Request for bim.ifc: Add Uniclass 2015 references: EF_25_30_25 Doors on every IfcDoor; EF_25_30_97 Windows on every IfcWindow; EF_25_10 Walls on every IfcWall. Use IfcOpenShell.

First a look at what the model holds.

```python
import ifcopenshell

model = ifcopenshell.open("bim.ifc")
print(model.schema)
print("classifications:", [c.Name for c in model.by_type("IfcClassification")])
for ifc_class in ("IfcDoor", "IfcRoof", "IfcStair", "IfcWall", "IfcWindow"):
    print(ifc_class, len(model.by_type(ifc_class)))
```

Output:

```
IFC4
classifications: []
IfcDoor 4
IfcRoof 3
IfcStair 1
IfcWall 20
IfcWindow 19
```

```python
import ifcopenshell
import ifcopenshell.api.classification

model = ifcopenshell.open("bim.ifc")

system = ifcopenshell.api.classification.add_classification(model, classification="Uniclass 2015")

codes = {
    "IfcDoor": ("EF_25_30_25", "Doors"),
    "IfcWindow": ("EF_25_30_97", "Windows"),
    "IfcWall": ("EF_25_10", "Walls"),
}
for ifc_class, (code, name) in codes.items():
    products = model.by_type(ifc_class)
    ifcopenshell.api.classification.add_reference(
        model, products=products, classification=system, identification=code, name=name
    )
    print(code, len(products))

model.write("bim_edited.ifc")
```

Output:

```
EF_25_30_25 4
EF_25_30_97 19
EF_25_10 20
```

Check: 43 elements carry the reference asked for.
